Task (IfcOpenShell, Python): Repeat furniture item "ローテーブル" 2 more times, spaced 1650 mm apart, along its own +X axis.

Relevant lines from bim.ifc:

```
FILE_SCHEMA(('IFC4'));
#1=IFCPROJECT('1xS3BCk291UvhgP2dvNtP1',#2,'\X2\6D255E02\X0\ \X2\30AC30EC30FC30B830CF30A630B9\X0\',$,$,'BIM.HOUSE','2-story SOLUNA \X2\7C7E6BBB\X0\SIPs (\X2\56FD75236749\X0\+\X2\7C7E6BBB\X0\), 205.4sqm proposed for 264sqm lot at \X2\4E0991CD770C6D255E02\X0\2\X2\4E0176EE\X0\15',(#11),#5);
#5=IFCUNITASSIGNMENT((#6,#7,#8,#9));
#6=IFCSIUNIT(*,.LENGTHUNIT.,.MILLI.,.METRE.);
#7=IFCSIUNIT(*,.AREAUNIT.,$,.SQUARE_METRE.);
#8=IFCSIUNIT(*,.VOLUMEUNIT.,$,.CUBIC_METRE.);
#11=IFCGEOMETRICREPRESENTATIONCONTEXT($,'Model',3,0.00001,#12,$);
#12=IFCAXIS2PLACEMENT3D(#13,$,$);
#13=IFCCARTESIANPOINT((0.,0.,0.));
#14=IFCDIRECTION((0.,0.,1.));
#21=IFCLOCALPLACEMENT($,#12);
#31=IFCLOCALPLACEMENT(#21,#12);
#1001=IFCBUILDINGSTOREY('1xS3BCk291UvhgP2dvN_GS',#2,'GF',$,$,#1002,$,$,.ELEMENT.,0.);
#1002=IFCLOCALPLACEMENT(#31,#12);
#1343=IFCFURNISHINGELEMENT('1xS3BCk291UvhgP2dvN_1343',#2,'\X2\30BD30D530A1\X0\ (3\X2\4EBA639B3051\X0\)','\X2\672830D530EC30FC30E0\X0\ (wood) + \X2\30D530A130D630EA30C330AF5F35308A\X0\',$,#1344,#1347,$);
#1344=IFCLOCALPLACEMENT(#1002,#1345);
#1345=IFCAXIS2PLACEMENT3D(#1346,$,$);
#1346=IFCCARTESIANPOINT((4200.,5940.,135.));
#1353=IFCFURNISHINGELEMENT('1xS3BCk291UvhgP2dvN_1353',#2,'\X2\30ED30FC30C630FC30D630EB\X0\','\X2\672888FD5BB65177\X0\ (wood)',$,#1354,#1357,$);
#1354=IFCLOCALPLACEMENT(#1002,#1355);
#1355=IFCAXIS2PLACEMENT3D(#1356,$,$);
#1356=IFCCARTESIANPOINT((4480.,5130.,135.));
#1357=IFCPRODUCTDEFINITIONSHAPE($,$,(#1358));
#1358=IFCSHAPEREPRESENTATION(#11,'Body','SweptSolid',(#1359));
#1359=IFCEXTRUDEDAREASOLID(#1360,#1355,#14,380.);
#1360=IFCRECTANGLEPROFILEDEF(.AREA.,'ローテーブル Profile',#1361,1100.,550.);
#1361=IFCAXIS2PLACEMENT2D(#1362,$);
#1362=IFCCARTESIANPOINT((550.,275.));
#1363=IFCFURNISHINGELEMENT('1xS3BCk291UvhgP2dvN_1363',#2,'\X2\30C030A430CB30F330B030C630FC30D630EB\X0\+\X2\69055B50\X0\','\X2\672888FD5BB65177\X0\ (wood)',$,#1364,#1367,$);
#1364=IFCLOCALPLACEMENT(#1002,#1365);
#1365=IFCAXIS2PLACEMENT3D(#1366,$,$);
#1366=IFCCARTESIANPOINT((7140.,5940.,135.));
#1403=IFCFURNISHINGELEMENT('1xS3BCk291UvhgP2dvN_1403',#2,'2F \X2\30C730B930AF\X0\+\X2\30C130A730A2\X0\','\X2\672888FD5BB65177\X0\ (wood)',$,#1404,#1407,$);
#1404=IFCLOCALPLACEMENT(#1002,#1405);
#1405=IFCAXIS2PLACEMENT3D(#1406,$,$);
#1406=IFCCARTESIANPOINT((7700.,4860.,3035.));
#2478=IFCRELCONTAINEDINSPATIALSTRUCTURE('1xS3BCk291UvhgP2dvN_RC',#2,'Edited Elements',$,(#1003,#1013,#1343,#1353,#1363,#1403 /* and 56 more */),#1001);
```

```python
import ifcopenshell
import ifcopenshell.api.geometry
import ifcopenshell.api.root
import ifcopenshell.util.element
import ifcopenshell.util.placement
import ifcopenshell.util.unit

model = ifcopenshell.open("bim.ifc")
unit_scale = ifcopenshell.util.unit.calculate_unit_scale(model)


def reuse_history(source, copy):
    """copy_class also copies each property set's owner history, people and application; keep the originals."""
    for rel in copy.IsDefinedBy:
        if rel.is_a("IfcRelDefinesByProperties") and (history := rel.RelatingPropertyDefinition.OwnerHistory):
            rel.RelatingPropertyDefinition.OwnerHistory = source.OwnerHistory
            ifcopenshell.util.element.remove_deep2(model, history)


source = model.by_guid("1xS3BCk291UvhgP2dvN_1353")
base = ifcopenshell.util.placement.get_local_placement(source.ObjectPlacement)
step = base[:3, 0] * 1.65 / unit_scale

for i in range(1, 3):
    copy = ifcopenshell.api.root.copy_class(model, product=source)
    copy.Representation = ifcopenshell.util.element.copy_deep(
        model, source.Representation, exclude=["IfcGeometricRepresentationContext", "IfcRepresentationMap"]
    )
    reuse_history(source, copy)
    matrix = base.copy()
    matrix[:3, 3] += i * step
    print("added at", matrix[:3, 3].round(3) + 0.0)
    ifcopenshell.api.geometry.edit_object_placement(model, product=copy, matrix=matrix, is_si=False)

model.write("bim-out.ifc")
```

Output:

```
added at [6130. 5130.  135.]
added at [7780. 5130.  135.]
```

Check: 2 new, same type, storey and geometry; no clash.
